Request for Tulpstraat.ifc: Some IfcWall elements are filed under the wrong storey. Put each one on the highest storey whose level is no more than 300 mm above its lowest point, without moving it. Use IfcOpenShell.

First a look at what the model holds.

```python
import ifcopenshell
import ifcopenshell.util.element
import ifcopenshell.util.placement

model = ifcopenshell.open("Tulpstraat.ifc")
print(model.schema)
for storey in model.by_type("IfcBuildingStorey"):
    level = ifcopenshell.util.placement.get_storey_elevation(storey)
    count = sum(e.is_a("IfcWall") for e in ifcopenshell.util.element.get_contained(storey))
    print(storey.id(), storey.Name, round(level, 3), count, sep=" | ")
```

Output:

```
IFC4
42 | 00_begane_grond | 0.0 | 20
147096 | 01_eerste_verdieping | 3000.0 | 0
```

```python
import ifcopenshell
import ifcopenshell.api.spatial
import ifcopenshell.geom
import ifcopenshell.util.element
import ifcopenshell.util.placement
import ifcopenshell.util.shape
import ifcopenshell.util.unit

model = ifcopenshell.open("Tulpstraat.ifc")
unit_scale = ifcopenshell.util.unit.calculate_unit_scale(model)
settings = ifcopenshell.geom.settings()

levels = sorted(
    ((ifcopenshell.util.placement.get_storey_elevation(s) * unit_scale, s) for s in model.by_type("IfcBuildingStorey")),
    key=lambda pair: pair[0],
)

for e in model.by_type("IfcWall"):
    current = e.ContainedInStructure[0].RelatingStructure if e.ContainedInStructure else None
    if current is None or not current.is_a("IfcBuildingStorey"):
        continue
    shape = ifcopenshell.geom.create_shape(settings, e)
    bottom = ifcopenshell.util.shape.get_shape_bottom_elevation(shape, shape.geometry)
    below = [s for level, s in levels if level <= bottom + 0.3]
    storey = below[-1] if below else levels[0][1]
    if storey != current:
        # assign_container keeps the world position.
        ifcopenshell.api.spatial.assign_container(model, products=[e], relating_structure=storey)
        print(e.id(), current.Name, "->", storey.Name)

model.write("Tulpstraat-out.ifc")
```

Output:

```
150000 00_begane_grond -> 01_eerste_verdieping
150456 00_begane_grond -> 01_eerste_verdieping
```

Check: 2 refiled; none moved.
